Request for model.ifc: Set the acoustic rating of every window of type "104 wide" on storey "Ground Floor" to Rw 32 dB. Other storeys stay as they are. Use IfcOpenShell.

First a look at what the model holds.

```python
import ifcopenshell
import ifcopenshell.util.element

model = ifcopenshell.open("model.ifc")
print(model.schema)
storey = next(s for s in model.by_type("IfcBuildingStorey") if s.Name == "Ground Floor")
windows = [e for e in ifcopenshell.util.element.get_decomposition(storey) if e.is_a("IfcWindow")]
seen = {}
for e in windows:
    element_type = ifcopenshell.util.element.get_type(e)
    key = (element_type.Name if element_type != e and element_type else None, ifcopenshell.util.element.get_pset(e, "Pset_WindowCommon", "AcousticRating"))
    seen[key] = seen.get(key, 0) + 1
for (name, value), count in sorted(seen.items(), key=str):
    print(count, "x", name, "|", value)
```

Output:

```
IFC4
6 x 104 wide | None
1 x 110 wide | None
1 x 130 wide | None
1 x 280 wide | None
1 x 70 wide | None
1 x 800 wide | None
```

```python
import ifcopenshell
import ifcopenshell.api.pset
import ifcopenshell.util.element

model = ifcopenshell.open("model.ifc")

storey = next(s for s in model.by_type("IfcBuildingStorey") if s.Name == "Ground Floor")
windows = [e for e in ifcopenshell.util.element.get_decomposition(storey) if e.is_a("IfcWindow")]

count = 0
for e in windows:
    element_type = ifcopenshell.util.element.get_type(e)
    if element_type in (None, e) or element_type.Name != "104 wide":
        continue
    # add_pset returns the element's existing set when there is one.
    pset = ifcopenshell.api.pset.add_pset(model, product=e, name="Pset_WindowCommon")
    ifcopenshell.api.pset.edit_pset(model, pset=pset, properties={"AcousticRating": "Rw 32 dB"})
    count += 1

print(count, "windows updated")

model.write("model_updated.ifc")
```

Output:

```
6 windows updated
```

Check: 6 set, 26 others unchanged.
